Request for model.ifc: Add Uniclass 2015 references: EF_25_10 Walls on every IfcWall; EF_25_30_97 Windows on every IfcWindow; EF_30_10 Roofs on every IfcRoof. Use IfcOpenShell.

First a look at what the model holds.

```python
import ifcopenshell

model = ifcopenshell.open("model.ifc")
print(model.schema)
print("classifications:", [c.Name for c in model.by_type("IfcClassification")])
for ifc_class in ("IfcDoor", "IfcRoof", "IfcStair", "IfcWall", "IfcWindow"):
    print(ifc_class, len(model.by_type(ifc_class)))
```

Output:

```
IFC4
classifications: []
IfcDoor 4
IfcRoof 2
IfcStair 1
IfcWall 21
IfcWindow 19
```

```python
import ifcopenshell
import ifcopenshell.api.classification

model = ifcopenshell.open("model.ifc")

system = ifcopenshell.api.classification.add_classification(model, classification="Uniclass 2015")

codes = {
    "IfcWall": ("EF_25_10", "Walls"),
    "IfcWindow": ("EF_25_30_97", "Windows"),
    "IfcRoof": ("EF_30_10", "Roofs"),
}
for ifc_class, (code, name) in codes.items():
    products = model.by_type(ifc_class)
    ifcopenshell.api.classification.add_reference(
        model, products=products, classification=system, identification=code, name=name
    )
    print(code, len(products))

model.write("model_rev.ifc")
```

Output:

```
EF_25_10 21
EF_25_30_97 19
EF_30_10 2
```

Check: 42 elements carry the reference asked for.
